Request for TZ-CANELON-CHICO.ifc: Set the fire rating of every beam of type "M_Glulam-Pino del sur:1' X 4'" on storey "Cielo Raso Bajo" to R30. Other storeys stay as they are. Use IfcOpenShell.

First a look at what the model holds.

```python
import ifcopenshell
import ifcopenshell.util.element

model = ifcopenshell.open("TZ-CANELON-CHICO.ifc")
print(model.schema)
storey = next(s for s in model.by_type("IfcBuildingStorey") if s.Name == "Cielo Raso Bajo")
beams = [e for e in ifcopenshell.util.element.get_decomposition(storey) if e.is_a("IfcBeam")]
seen = {}
for e in beams:
    element_type = ifcopenshell.util.element.get_type(e)
    key = (element_type.Name if element_type != e and element_type else None, ifcopenshell.util.element.get_pset(e, "Pset_BeamCommon", "FireRating"))
    seen[key] = seen.get(key, 0) + 1
for (name, value), count in sorted(seen.items(), key=str):
    print(count, "x", name, "|", value)
```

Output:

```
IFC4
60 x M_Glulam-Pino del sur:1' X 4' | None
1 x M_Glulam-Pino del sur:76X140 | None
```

```python
import ifcopenshell
import ifcopenshell.api.pset
import ifcopenshell.util.element

model = ifcopenshell.open("TZ-CANELON-CHICO.ifc")

storey = next(s for s in model.by_type("IfcBuildingStorey") if s.Name == "Cielo Raso Bajo")
beams = [e for e in ifcopenshell.util.element.get_decomposition(storey) if e.is_a("IfcBeam")]

count = 0
for e in beams:
    element_type = ifcopenshell.util.element.get_type(e)
    if element_type in (None, e) or element_type.Name != "M_Glulam-Pino del sur:1' X 4'":
        continue
    # add_pset returns the element's existing set when there is one.
    pset = ifcopenshell.api.pset.add_pset(model, product=e, name="Pset_BeamCommon")
    ifcopenshell.api.pset.edit_pset(model, pset=pset, properties={"FireRating": "R30"})
    count += 1

print(count, "beams updated")

model.write("TZ-CANELON-CHICO_rev.ifc")
```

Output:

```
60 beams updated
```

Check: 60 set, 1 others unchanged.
